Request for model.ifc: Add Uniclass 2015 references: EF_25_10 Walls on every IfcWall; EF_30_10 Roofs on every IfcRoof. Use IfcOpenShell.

First a look at what the model holds.

```python
import ifcopenshell

model = ifcopenshell.open("model.ifc")
print(model.schema)
print("classifications:", [c.Name for c in model.by_type("IfcClassification")])
for ifc_class in ("IfcDoor", "IfcRoof", "IfcStair", "IfcWall", "IfcWindow"):
    print(ifc_class, len(model.by_type(ifc_class)))
```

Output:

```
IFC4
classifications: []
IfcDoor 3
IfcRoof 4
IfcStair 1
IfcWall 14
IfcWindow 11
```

```python
import ifcopenshell
import ifcopenshell.api.classification

model = ifcopenshell.open("model.ifc")

system = ifcopenshell.api.classification.add_classification(model, classification="Uniclass 2015")

codes = {
    "IfcWall": ("EF_25_10", "Walls"),
    "IfcRoof": ("EF_30_10", "Roofs"),
}
for ifc_class, (code, name) in codes.items():
    products = model.by_type(ifc_class)
    ifcopenshell.api.classification.add_reference(
        model, products=products, classification=system, identification=code, name=name
    )
    print(code, len(products))

model.write("model_edited.ifc")
```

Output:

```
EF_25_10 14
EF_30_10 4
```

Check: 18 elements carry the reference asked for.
